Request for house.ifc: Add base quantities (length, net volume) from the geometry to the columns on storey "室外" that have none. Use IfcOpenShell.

First a look at what the model holds.

```python
import ifcopenshell
import ifcopenshell.util.element
import ifcopenshell.util.unit

model = ifcopenshell.open("house.ifc")
print(model.schema)
for unit_type in ("LENGTHUNIT", "AREAUNIT", "VOLUMEUNIT"):
    print(unit_type, ifcopenshell.util.unit.calculate_unit_scale(model, unit_type))
storey = next(s for s in model.by_type("IfcBuildingStorey") if s.Name == "室外")
columns = [e for e in ifcopenshell.util.element.get_decomposition(storey) if e.is_a("IfcColumn")]
for e in sorted(columns, key=lambda e: e.id()):
    print(e.id(), e.is_a(), e.Name, list(ifcopenshell.util.element.get_psets(e, qtos_only=True)), sep=" | ")
```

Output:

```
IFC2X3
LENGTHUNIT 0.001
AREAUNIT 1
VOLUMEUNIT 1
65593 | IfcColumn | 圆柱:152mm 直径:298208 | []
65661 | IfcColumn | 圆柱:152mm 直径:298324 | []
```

```python
import ifcopenshell
import ifcopenshell.api.pset
import ifcopenshell.geom
import ifcopenshell.util.element
import ifcopenshell.util.shape
import ifcopenshell.util.unit

model = ifcopenshell.open("house.ifc")
unit_scale = ifcopenshell.util.unit.calculate_unit_scale(model)
volume_scale = ifcopenshell.util.unit.calculate_unit_scale(model, "VOLUMEUNIT")
settings = ifcopenshell.geom.settings()

storey = next(s for s in model.by_type("IfcBuildingStorey") if s.Name == "室外")
columns = [e for e in ifcopenshell.util.element.get_decomposition(storey) if e.is_a("IfcColumn")]

for e in sorted(columns, key=lambda e: e.id()):
    if ifcopenshell.util.element.get_psets(e, qtos_only=True, should_inherit=False):
        continue
    # Geometry comes back in metres, in the element's own axes.
    shape = ifcopenshell.geom.create_shape(settings, e)
    values = {
        "Length": ifcopenshell.util.shape.get_z(shape.geometry) / unit_scale,
        "NetVolume": ifcopenshell.util.shape.get_volume(shape.geometry) / volume_scale,
    }
    qto = ifcopenshell.api.pset.add_qto(model, product=e, name="BaseQuantities")
    ifcopenshell.api.pset.edit_qto(model, qto=qto, properties=values)
    print(e.id(), {k: round(v, 3) for k, v in values.items()})

model.write("house_updated.ifc")
```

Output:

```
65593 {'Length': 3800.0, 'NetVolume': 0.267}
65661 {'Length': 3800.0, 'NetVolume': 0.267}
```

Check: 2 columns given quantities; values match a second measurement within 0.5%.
